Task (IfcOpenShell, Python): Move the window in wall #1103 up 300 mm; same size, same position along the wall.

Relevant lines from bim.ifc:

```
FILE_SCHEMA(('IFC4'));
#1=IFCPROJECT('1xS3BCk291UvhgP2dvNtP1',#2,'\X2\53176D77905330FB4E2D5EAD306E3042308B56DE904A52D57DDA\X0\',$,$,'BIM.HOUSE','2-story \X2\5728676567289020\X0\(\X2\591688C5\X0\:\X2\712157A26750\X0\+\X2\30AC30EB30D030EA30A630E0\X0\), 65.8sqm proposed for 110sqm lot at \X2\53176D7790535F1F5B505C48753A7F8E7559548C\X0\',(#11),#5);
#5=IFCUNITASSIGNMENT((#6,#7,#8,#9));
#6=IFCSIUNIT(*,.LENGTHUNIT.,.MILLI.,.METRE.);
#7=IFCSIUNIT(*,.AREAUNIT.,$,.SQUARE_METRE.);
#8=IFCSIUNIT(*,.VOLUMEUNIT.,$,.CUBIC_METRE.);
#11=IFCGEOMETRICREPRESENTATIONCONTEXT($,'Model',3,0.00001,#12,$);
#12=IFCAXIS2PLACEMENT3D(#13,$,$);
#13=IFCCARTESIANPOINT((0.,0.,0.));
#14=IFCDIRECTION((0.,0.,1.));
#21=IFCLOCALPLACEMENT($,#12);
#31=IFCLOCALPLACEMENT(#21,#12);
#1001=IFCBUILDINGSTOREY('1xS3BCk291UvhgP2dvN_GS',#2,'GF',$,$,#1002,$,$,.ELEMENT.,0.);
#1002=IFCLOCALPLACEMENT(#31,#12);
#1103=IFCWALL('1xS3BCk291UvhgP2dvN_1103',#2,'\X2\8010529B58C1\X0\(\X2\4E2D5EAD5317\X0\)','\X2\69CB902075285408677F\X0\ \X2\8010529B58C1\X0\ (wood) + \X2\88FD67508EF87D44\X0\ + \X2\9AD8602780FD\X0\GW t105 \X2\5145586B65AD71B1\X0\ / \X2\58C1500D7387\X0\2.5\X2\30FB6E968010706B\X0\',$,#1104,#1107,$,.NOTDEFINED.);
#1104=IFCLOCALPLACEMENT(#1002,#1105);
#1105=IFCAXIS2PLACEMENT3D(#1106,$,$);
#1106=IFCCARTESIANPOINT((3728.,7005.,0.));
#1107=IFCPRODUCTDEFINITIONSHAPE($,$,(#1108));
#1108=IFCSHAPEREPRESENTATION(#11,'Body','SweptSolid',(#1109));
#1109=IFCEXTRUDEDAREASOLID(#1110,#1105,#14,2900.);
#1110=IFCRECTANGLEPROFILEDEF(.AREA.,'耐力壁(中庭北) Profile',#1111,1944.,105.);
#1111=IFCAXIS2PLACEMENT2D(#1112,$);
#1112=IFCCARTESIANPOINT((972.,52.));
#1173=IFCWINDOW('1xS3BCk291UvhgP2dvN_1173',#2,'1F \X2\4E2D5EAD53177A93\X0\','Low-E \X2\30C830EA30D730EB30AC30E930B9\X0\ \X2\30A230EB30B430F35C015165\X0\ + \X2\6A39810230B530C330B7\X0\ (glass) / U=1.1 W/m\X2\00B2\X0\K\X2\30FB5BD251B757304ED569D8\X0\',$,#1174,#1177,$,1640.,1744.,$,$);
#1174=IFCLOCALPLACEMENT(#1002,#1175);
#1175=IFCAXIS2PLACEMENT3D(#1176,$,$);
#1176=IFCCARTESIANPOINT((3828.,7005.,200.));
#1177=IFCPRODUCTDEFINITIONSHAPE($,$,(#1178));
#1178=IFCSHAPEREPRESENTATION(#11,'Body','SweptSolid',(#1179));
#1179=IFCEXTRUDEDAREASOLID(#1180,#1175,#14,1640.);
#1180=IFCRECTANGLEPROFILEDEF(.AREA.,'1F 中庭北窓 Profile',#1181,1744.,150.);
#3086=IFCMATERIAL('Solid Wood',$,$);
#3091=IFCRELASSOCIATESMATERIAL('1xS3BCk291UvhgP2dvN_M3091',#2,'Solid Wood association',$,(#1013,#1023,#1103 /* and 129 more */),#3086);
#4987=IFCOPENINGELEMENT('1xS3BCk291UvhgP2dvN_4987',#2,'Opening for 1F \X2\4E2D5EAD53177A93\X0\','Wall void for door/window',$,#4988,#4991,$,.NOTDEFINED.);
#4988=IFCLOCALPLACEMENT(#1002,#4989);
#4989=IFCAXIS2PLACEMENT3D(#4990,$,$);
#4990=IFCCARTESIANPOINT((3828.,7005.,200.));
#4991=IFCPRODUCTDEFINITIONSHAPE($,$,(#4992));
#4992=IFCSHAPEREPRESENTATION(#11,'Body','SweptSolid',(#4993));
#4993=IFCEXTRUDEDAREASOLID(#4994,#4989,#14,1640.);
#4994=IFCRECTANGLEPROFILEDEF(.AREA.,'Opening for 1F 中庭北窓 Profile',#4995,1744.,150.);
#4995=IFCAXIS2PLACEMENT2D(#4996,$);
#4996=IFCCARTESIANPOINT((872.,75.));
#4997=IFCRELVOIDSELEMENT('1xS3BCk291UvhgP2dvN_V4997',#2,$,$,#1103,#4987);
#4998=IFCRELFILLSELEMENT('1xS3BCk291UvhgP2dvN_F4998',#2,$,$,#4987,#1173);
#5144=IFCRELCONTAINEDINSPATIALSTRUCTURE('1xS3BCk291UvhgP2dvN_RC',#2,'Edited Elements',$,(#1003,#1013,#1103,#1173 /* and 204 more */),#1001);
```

```python
import numpy as np
import ifcopenshell
import ifcopenshell.api.geometry
import ifcopenshell.util.placement
import ifcopenshell.util.unit

model = ifcopenshell.open("bim.ifc")
unit_scale = ifcopenshell.util.unit.calculate_unit_scale(model)

window = model.by_guid("1xS3BCk291UvhgP2dvN_1173")
opening = window.FillsVoids[0].RelatingOpeningElement
dz = 0.3 / unit_scale

shift = np.array([0.0, 0.0, dz])
# The window is not placed relative to its opening, so move both.
for product in (opening, window):
    matrix = ifcopenshell.util.placement.get_local_placement(product.ObjectPlacement)
    matrix[:3, 3] += shift
    ifcopenshell.api.geometry.edit_object_placement(model, product=product, matrix=matrix, is_si=False)

print(f"moved by {dz * unit_scale:+.3f} m")

model.write("bim_rev.ifc")
```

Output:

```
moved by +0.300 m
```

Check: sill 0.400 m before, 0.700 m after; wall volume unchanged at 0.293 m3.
